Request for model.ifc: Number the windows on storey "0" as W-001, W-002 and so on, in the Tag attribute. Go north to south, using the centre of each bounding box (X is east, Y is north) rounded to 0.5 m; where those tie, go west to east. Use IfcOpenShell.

First a look at what the model holds.

```python
import ifcopenshell
import ifcopenshell.util.element
import ifcopenshell.util.placement

model = ifcopenshell.open("model.ifc")
print(model.schema)
storey = next(s for s in model.by_type("IfcBuildingStorey") if s.Name == "0")
windows = [e for e in ifcopenshell.util.element.get_decomposition(storey) if e.is_a("IfcWindow")]
for e in sorted(windows, key=lambda e: e.id()):
    origin = ifcopenshell.util.placement.get_local_placement(e.ObjectPlacement)[:3, 3]
    print(e.id(), e.Tag, e.Name, origin.round(2) + 0.0, sep=" | ")
```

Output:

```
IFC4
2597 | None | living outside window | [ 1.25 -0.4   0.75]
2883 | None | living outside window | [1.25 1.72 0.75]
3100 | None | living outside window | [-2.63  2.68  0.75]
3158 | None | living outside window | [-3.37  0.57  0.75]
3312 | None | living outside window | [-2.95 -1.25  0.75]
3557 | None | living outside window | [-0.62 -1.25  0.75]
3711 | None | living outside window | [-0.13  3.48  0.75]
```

```python
import ifcopenshell
import ifcopenshell.geom
import ifcopenshell.util.element
import ifcopenshell.util.shape

model = ifcopenshell.open("model.ifc")
settings = ifcopenshell.geom.settings()
settings.set("use-world-coords", True)


def centre(element):
    shape = ifcopenshell.geom.create_shape(settings, element)
    return ifcopenshell.util.shape.get_bbox_centroid(shape.geometry)


storey = next(s for s in model.by_type("IfcBuildingStorey") if s.Name == "0")
windows = [e for e in ifcopenshell.util.element.get_decomposition(storey) if e.is_a("IfcWindow")]

# Insertion points can sit at a corner or the storey origin, so sort by the geometry (in metres).
centres = {e: centre(e) for e in windows}
windows.sort(key=lambda e: (-round(centres[e][1] / 0.5), centres[e][0]))

for i, e in enumerate(windows, start=1):
    number = f"W-0{i:02d}"
    e.Tag = number
    print(e.id(), number)

model.write("model_rev.ifc")
```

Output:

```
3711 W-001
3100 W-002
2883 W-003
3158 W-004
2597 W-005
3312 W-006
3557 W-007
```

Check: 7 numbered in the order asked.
